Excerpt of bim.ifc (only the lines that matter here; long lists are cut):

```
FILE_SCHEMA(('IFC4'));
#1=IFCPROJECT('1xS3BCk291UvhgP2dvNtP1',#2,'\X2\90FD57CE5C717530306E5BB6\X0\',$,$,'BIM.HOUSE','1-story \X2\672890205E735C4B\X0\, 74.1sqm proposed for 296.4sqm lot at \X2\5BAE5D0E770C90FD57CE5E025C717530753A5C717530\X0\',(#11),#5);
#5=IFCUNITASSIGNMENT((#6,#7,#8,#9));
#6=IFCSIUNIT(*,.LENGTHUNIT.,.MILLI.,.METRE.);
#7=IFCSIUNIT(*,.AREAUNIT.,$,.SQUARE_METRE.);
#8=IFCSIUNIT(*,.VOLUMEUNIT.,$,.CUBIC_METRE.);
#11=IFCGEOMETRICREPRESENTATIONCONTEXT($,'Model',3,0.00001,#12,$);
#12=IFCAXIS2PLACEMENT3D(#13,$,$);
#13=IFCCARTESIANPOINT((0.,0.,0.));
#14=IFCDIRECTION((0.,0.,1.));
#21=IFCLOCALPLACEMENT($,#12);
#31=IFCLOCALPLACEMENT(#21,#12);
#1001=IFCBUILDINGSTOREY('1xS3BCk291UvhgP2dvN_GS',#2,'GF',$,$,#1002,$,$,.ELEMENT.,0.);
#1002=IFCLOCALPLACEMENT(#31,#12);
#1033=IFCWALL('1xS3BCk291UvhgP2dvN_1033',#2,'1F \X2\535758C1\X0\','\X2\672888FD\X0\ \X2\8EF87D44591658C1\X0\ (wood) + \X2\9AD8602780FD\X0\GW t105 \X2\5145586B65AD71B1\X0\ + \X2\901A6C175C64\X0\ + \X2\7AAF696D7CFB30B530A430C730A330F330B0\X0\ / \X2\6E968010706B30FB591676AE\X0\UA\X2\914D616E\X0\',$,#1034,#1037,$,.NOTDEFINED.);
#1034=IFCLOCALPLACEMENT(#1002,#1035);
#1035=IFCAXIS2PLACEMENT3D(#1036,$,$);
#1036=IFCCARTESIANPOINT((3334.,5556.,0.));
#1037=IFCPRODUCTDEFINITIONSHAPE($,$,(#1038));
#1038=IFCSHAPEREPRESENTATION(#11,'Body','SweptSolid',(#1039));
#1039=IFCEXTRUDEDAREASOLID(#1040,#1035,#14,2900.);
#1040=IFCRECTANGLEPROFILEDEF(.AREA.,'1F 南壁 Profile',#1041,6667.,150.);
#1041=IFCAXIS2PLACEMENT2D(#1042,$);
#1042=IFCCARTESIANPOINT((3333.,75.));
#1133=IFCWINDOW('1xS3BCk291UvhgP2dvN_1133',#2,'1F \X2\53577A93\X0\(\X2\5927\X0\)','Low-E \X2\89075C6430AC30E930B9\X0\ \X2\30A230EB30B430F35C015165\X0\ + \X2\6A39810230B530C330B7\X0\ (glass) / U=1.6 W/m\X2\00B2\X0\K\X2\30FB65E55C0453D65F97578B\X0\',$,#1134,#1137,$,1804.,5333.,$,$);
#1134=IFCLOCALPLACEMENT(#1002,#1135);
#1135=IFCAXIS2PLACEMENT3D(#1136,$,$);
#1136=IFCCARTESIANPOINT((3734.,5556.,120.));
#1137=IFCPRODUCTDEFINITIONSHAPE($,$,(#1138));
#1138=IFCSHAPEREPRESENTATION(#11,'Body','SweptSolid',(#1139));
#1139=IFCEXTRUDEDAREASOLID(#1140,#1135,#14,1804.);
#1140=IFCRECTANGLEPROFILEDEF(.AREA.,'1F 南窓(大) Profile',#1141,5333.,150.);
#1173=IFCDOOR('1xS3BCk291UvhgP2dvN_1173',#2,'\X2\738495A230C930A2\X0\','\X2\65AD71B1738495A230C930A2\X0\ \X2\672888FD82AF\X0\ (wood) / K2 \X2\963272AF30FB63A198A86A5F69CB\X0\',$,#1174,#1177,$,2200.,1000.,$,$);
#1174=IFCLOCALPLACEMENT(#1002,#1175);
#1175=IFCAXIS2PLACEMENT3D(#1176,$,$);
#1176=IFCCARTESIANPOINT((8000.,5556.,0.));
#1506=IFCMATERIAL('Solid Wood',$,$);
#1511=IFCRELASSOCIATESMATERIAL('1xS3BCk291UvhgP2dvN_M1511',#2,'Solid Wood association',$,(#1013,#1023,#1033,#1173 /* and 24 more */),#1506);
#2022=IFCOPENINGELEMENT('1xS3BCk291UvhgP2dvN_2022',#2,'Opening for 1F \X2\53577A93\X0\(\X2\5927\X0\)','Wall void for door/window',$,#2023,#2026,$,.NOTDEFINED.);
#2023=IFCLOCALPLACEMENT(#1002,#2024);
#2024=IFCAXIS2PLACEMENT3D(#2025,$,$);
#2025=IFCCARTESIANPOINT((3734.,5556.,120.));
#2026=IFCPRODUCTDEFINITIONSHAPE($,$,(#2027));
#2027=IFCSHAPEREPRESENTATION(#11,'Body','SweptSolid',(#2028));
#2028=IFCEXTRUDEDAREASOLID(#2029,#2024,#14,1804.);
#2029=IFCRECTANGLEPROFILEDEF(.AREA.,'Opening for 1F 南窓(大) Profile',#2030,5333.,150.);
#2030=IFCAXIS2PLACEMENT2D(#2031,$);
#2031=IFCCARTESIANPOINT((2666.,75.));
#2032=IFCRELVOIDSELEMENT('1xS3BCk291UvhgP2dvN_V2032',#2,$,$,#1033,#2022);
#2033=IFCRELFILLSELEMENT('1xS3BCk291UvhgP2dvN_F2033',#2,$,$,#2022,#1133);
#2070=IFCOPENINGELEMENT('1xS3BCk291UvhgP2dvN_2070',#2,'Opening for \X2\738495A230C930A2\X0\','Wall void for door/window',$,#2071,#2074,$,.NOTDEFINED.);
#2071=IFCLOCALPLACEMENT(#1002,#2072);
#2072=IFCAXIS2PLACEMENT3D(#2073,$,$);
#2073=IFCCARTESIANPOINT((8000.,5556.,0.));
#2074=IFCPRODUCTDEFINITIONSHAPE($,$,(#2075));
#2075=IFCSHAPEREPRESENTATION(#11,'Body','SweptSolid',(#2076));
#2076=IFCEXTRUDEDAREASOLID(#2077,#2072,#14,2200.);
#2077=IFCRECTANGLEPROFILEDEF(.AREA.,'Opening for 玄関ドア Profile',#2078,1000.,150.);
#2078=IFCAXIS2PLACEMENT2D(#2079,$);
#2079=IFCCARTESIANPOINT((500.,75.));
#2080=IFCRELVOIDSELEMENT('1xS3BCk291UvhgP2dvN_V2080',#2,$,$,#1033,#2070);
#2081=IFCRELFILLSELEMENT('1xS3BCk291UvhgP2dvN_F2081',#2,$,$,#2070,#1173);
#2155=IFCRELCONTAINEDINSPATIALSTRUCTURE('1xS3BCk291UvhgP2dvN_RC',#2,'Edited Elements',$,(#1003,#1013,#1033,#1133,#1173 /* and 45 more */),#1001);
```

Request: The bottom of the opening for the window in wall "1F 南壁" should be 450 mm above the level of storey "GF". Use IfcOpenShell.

```python
import numpy as np
import ifcopenshell
import ifcopenshell.api.geometry
import ifcopenshell.geom
import ifcopenshell.util.element
import ifcopenshell.util.placement
import ifcopenshell.util.shape
import ifcopenshell.util.unit

model = ifcopenshell.open("bim.ifc")
unit_scale = ifcopenshell.util.unit.calculate_unit_scale(model)

window = model.by_guid("1xS3BCk291UvhgP2dvN_1133")
opening = window.FillsVoids[0].RelatingOpeningElement
storey = ifcopenshell.util.element.get_container(window, ifc_class="IfcBuildingStorey")
level = ifcopenshell.util.placement.get_local_placement(storey.ObjectPlacement)[2, 3]

# The opening's origin need not be at the sill, so measure its lowest point.
shape = ifcopenshell.geom.create_shape(ifcopenshell.geom.settings(), opening)
bottom = ifcopenshell.util.shape.get_shape_bottom_elevation(shape, shape.geometry) / unit_scale
dz = level + 450.0 - bottom

shift = np.array([0.0, 0.0, dz])
# The window is not placed relative to its opening, so move both.
for product in (opening, window):
    matrix = ifcopenshell.util.placement.get_local_placement(product.ObjectPlacement)
    matrix[:3, 3] += shift
    ifcopenshell.api.geometry.edit_object_placement(model, product=product, matrix=matrix, is_si=False)

print(f"moved by {dz * unit_scale:+.3f} m")

model.write("bim_updated.ifc")
```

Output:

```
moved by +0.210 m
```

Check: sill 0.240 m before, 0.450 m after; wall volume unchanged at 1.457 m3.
